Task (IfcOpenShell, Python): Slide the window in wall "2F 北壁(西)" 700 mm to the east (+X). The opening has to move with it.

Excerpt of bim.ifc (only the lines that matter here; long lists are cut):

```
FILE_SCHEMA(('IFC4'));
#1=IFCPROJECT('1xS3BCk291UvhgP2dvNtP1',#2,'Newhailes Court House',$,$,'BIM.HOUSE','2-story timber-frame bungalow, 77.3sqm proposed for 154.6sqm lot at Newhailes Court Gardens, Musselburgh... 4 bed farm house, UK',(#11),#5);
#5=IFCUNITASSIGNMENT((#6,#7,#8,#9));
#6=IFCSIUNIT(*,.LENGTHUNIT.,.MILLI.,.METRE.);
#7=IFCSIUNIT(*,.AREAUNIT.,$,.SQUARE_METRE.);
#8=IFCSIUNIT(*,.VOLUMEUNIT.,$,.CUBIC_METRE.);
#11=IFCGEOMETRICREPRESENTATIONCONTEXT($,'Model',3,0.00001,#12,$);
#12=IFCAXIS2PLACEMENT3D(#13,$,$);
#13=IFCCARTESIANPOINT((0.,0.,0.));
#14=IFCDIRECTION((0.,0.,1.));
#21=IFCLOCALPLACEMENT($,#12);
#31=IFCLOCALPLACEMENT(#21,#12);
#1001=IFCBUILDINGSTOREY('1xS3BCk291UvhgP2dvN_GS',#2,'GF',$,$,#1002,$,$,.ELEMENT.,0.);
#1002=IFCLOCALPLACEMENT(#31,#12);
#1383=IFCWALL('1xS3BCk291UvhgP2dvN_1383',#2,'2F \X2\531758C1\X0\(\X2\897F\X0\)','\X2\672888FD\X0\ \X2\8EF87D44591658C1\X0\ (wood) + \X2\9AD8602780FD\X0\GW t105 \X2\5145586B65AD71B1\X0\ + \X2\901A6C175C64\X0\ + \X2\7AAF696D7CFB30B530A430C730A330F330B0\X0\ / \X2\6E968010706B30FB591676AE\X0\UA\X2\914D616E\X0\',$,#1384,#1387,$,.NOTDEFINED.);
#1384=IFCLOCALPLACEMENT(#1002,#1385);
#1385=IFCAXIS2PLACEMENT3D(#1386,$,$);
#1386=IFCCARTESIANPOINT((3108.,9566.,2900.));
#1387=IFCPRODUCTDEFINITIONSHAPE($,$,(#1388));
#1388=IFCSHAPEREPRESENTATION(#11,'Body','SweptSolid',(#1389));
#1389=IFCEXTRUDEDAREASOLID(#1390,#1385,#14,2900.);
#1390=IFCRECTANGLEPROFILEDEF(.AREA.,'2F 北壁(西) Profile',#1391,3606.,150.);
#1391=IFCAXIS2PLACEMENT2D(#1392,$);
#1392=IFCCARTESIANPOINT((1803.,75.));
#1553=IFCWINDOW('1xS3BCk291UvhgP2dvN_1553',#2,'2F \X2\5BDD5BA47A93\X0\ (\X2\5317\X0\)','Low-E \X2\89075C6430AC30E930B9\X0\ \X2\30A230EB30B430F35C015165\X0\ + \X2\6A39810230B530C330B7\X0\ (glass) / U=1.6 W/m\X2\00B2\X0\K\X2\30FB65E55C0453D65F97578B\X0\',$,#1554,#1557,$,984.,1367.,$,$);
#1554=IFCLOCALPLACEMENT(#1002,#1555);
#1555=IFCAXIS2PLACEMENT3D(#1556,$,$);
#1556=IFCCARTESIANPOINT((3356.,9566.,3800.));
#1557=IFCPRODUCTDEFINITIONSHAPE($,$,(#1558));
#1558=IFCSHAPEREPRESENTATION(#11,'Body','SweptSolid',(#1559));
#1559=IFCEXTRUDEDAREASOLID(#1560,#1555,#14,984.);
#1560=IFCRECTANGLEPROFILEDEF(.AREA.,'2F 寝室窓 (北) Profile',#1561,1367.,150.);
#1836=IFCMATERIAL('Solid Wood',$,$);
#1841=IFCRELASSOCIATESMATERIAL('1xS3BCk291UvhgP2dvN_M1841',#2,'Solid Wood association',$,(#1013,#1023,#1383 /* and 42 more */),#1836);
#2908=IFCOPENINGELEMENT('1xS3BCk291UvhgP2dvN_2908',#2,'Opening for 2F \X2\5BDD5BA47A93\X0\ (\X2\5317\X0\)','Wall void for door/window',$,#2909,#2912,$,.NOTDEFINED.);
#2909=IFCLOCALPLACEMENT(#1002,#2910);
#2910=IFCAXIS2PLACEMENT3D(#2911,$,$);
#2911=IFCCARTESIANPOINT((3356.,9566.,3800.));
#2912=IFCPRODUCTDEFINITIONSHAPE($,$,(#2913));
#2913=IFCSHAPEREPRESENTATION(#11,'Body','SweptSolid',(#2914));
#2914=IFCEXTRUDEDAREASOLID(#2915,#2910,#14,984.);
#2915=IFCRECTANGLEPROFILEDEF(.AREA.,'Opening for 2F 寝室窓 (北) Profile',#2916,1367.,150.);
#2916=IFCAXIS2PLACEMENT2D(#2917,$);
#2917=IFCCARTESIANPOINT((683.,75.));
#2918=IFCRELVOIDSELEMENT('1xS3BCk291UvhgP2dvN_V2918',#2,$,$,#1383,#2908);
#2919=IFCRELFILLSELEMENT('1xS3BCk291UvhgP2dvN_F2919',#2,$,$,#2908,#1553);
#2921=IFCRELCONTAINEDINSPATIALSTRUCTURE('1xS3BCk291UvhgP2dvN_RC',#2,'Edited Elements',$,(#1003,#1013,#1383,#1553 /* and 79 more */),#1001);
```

```python
import ifcopenshell
import ifcopenshell.api.geometry
import ifcopenshell.util.placement
import ifcopenshell.util.unit

model = ifcopenshell.open("bim.ifc")
unit_scale = ifcopenshell.util.unit.calculate_unit_scale(model)

window = model.by_guid("1xS3BCk291UvhgP2dvN_1553")
opening = window.FillsVoids[0].RelatingOpeningElement
wall = opening.VoidsElements[0].RelatingBuildingElement

wall_matrix = ifcopenshell.util.placement.get_local_placement(wall.ObjectPlacement)
shift = wall_matrix[:3, 0] * 0.7 / unit_scale
before = ifcopenshell.util.placement.get_local_placement(window.ObjectPlacement)[:3, 3].copy()

# The window is not placed relative to its opening, so move both.
for product in (opening, window):
    matrix = ifcopenshell.util.placement.get_local_placement(product.ObjectPlacement)
    matrix[:3, 3] += shift
    ifcopenshell.api.geometry.edit_object_placement(model, product=product, matrix=matrix, is_si=False)

after = ifcopenshell.util.placement.get_local_placement(window.ObjectPlacement)[:3, 3]
print("window moved by", (after - before).round(3) + 0.0)

model.write("bim_rev.ifc")
```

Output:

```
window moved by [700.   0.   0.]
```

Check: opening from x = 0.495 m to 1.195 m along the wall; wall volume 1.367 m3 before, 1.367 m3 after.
